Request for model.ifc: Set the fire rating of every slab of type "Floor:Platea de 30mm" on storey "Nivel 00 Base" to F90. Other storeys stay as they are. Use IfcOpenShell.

First a look at what the model holds.

```python
import ifcopenshell
import ifcopenshell.util.element

model = ifcopenshell.open("model.ifc")
print(model.schema)
storey = next(s for s in model.by_type("IfcBuildingStorey") if s.Name == "Nivel 00 Base")
slabs = [e for e in ifcopenshell.util.element.get_decomposition(storey) if e.is_a("IfcSlab")]
seen = {}
for e in slabs:
    element_type = ifcopenshell.util.element.get_type(e)
    key = (element_type.Name if element_type != e and element_type else None, ifcopenshell.util.element.get_pset(e, "Pset_SlabCommon", "FireRating"))
    seen[key] = seen.get(key, 0) + 1
for (name, value), count in sorted(seen.items(), key=str):
    print(count, "x", name, "|", value)
```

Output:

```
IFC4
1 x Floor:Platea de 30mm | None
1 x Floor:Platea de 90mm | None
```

```python
import ifcopenshell
import ifcopenshell.api.pset
import ifcopenshell.util.element

model = ifcopenshell.open("model.ifc")

storey = next(s for s in model.by_type("IfcBuildingStorey") if s.Name == "Nivel 00 Base")
slabs = [e for e in ifcopenshell.util.element.get_decomposition(storey) if e.is_a("IfcSlab")]

count = 0
for e in slabs:
    element_type = ifcopenshell.util.element.get_type(e)
    if element_type in (None, e) or element_type.Name != "Floor:Platea de 30mm":
        continue
    # add_pset returns the element's existing set when there is one.
    pset = ifcopenshell.api.pset.add_pset(model, product=e, name="Pset_SlabCommon")
    ifcopenshell.api.pset.edit_pset(model, pset=pset, properties={"FireRating": "F90"})
    count += 1

print(count, "slabs updated")

model.write("model-out.ifc")
```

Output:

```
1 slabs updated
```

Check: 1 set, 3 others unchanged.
